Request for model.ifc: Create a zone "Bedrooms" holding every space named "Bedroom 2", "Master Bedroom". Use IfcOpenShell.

First a look at what the model holds.

```python
import ifcopenshell

model = ifcopenshell.open("model.ifc")
print(model.schema)
seen = {}
for space in model.by_type("IfcSpace"):
    seen[space.LongName] = seen.get(space.LongName, 0) + 1
for name, count in sorted(seen.items(), key=str):
    print(count, "x", name)
print("zones:", [z.Name for z in model.by_type("IfcZone")][:20])
```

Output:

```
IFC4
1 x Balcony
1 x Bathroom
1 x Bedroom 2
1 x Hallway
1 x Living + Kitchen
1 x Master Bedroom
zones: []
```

```python
import ifcopenshell
import ifcopenshell.api.group
import ifcopenshell.api.root

model = ifcopenshell.open("model.ifc")

names = {"Bedroom 2", "Master Bedroom"}
spaces = [s for s in model.by_type("IfcSpace") if s.LongName in names]

zone = ifcopenshell.api.root.create_entity(model, ifc_class="IfcZone", name="Bedrooms")
ifcopenshell.api.group.assign_group(model, products=spaces, group=zone)
print(len(spaces), "spaces in", zone.Name)

model.write("model_rev.ifc")
```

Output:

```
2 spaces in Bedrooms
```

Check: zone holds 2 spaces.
